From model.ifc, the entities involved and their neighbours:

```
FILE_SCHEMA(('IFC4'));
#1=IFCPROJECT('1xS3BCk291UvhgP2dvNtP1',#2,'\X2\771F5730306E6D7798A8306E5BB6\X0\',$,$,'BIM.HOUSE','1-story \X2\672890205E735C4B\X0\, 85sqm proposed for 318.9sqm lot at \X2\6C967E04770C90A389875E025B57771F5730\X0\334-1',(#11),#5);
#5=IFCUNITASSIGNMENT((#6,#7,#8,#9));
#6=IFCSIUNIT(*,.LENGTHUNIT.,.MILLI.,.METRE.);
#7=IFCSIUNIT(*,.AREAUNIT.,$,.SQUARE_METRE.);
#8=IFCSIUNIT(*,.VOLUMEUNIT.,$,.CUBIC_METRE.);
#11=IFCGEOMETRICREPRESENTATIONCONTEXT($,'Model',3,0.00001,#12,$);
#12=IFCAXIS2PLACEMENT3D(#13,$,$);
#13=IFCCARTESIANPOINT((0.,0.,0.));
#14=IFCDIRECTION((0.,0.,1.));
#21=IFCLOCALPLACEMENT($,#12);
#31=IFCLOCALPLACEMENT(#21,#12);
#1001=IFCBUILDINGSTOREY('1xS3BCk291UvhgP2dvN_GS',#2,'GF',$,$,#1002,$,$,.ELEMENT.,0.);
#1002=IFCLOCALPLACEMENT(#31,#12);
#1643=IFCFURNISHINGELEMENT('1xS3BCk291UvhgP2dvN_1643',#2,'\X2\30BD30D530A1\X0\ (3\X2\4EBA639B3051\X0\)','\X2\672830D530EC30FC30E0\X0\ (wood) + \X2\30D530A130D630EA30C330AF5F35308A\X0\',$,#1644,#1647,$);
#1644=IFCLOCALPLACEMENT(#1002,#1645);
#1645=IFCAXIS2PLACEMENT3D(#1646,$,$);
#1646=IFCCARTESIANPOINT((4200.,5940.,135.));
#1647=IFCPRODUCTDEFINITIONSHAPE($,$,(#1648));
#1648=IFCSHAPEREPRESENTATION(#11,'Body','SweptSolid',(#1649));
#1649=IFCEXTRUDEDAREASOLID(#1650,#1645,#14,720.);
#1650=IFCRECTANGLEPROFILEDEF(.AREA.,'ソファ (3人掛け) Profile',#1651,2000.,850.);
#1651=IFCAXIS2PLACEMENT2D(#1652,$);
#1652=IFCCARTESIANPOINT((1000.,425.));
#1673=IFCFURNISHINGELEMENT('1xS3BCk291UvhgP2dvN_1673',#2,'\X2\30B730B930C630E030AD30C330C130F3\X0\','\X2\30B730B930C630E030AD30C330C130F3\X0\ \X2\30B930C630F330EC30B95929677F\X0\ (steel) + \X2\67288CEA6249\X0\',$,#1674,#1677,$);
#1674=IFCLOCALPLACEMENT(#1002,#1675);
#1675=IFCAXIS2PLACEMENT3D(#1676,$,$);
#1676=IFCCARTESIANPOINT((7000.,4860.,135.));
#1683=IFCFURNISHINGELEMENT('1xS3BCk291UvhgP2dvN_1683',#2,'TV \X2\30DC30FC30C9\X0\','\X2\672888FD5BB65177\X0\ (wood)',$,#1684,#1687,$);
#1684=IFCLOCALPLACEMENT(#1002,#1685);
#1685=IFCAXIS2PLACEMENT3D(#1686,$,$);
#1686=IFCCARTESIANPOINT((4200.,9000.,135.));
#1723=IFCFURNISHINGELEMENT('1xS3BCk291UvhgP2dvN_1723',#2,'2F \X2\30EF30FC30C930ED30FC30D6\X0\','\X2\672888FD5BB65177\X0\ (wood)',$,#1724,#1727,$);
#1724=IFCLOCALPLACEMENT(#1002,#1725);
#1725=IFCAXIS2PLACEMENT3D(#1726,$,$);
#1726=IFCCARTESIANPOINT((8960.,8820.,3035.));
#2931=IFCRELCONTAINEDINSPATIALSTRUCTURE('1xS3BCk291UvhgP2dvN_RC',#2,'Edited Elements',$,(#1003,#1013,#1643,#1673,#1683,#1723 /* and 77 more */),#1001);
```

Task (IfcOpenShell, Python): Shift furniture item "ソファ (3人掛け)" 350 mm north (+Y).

```python
import ifcopenshell
import ifcopenshell.api.geometry
import ifcopenshell.util.placement

model = ifcopenshell.open("model.ifc")

item = model.by_guid("1xS3BCk291UvhgP2dvN_1643")
matrix = ifcopenshell.util.placement.get_local_placement(item.ObjectPlacement)
matrix[1, 3] += 350.0
ifcopenshell.api.geometry.edit_object_placement(model, product=item, matrix=matrix, is_si=False)

print(ifcopenshell.util.placement.get_local_placement(item.ObjectPlacement).round(3) + 0.0)

model.write("model_rev.ifc")
```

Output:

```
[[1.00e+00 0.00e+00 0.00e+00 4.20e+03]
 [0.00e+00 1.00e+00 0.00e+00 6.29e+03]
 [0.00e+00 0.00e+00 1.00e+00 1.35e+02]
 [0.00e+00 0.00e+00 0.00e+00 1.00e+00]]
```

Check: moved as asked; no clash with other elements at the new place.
